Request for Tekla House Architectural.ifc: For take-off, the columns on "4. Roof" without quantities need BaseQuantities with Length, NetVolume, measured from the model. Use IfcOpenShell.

First a look at what the model holds.

```python
import ifcopenshell
import ifcopenshell.util.element
import ifcopenshell.util.unit

model = ifcopenshell.open("Tekla House Architectural.ifc")
print(model.schema)
for unit_type in ("LENGTHUNIT", "AREAUNIT", "VOLUMEUNIT"):
    print(unit_type, ifcopenshell.util.unit.calculate_unit_scale(model, unit_type))
storey = next(s for s in model.by_type("IfcBuildingStorey") if s.Name == "4. Roof")
columns = [e for e in ifcopenshell.util.element.get_decomposition(storey) if e.is_a("IfcColumn")]
for e in sorted(columns, key=lambda e: e.id()):
    print(e.id(), e.is_a(), e.Name, list(ifcopenshell.util.element.get_psets(e, qtos_only=True)), sep=" | ")
```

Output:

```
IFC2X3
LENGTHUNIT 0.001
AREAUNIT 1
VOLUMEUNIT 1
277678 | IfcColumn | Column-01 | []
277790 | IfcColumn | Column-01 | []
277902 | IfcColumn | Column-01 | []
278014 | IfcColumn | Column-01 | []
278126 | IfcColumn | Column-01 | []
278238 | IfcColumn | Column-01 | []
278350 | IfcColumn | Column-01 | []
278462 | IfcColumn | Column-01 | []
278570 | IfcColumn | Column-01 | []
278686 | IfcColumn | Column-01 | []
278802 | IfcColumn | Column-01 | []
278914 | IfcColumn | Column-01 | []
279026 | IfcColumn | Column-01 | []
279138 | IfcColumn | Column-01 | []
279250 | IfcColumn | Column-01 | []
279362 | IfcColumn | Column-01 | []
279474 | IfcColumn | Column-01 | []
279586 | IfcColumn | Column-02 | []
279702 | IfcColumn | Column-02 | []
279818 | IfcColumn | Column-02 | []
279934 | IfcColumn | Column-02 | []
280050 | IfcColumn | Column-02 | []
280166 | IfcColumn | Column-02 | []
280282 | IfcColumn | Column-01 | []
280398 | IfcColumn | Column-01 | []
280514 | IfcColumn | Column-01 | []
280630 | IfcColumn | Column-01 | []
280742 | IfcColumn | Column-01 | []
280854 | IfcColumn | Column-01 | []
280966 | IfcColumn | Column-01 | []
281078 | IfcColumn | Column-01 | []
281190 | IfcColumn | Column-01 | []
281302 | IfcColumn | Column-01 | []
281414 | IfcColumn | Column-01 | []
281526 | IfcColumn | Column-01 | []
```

```python
import ifcopenshell
import ifcopenshell.api.pset
import ifcopenshell.geom
import ifcopenshell.util.element
import ifcopenshell.util.shape
import ifcopenshell.util.unit

model = ifcopenshell.open("Tekla House Architectural.ifc")
unit_scale = ifcopenshell.util.unit.calculate_unit_scale(model)
volume_scale = ifcopenshell.util.unit.calculate_unit_scale(model, "VOLUMEUNIT")
settings = ifcopenshell.geom.settings()

storey = next(s for s in model.by_type("IfcBuildingStorey") if s.Name == "4. Roof")
columns = [e for e in ifcopenshell.util.element.get_decomposition(storey) if e.is_a("IfcColumn")]

for e in sorted(columns, key=lambda e: e.id()):
    if ifcopenshell.util.element.get_psets(e, qtos_only=True, should_inherit=False):
        continue
    # Geometry comes back in metres, in the element's own axes.
    shape = ifcopenshell.geom.create_shape(settings, e)
    values = {
        "Length": ifcopenshell.util.shape.get_z(shape.geometry) / unit_scale,
        "NetVolume": ifcopenshell.util.shape.get_volume(shape.geometry) / volume_scale,
    }
    qto = ifcopenshell.api.pset.add_qto(model, product=e, name="BaseQuantities")
    ifcopenshell.api.pset.edit_qto(model, qto=qto, properties=values)
    print(e.id(), {k: round(v, 3) for k, v in values.items()})

model.write("Tekla House Architectural_v2.ifc")
```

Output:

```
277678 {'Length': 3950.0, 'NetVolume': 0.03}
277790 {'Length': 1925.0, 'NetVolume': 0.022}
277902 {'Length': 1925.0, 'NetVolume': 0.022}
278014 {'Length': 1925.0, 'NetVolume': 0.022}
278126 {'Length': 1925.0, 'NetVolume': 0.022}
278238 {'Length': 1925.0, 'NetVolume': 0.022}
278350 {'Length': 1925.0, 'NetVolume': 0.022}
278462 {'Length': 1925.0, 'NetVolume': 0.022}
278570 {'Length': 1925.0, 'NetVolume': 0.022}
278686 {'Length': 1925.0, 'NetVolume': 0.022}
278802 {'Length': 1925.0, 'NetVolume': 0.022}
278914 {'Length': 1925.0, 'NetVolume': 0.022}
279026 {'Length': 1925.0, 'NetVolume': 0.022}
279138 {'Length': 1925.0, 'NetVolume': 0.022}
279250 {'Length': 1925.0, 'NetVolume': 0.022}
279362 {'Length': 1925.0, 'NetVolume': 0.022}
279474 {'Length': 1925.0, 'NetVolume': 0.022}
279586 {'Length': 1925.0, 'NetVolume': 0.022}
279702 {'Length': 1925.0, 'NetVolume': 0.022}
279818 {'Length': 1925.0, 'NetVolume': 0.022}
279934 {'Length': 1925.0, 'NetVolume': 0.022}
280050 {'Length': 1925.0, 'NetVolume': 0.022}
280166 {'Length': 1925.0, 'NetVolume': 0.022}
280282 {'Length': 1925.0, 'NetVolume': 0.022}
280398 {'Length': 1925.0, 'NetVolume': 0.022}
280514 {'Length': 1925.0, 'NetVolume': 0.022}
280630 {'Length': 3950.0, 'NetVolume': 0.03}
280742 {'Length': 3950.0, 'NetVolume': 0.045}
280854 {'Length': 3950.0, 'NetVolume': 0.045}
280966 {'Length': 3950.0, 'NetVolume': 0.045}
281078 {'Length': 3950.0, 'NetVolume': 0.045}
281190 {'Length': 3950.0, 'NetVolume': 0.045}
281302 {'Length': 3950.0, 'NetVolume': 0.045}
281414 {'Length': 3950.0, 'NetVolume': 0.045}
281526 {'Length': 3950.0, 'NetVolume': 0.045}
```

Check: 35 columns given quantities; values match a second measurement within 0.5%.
